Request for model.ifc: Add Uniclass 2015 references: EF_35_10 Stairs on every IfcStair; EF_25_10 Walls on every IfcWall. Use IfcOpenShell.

First a look at what the model holds.

```python
import ifcopenshell

model = ifcopenshell.open("model.ifc")
print(model.schema)
print("classifications:", [c.Name for c in model.by_type("IfcClassification")])
for ifc_class in ("IfcDoor", "IfcRoof", "IfcStair", "IfcWall", "IfcWindow"):
    print(ifc_class, len(model.by_type(ifc_class)))
```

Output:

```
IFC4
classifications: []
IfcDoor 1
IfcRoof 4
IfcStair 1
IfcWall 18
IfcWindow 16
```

```python
import ifcopenshell
import ifcopenshell.api.classification

model = ifcopenshell.open("model.ifc")

system = ifcopenshell.api.classification.add_classification(model, classification="Uniclass 2015")

codes = {
    "IfcStair": ("EF_35_10", "Stairs"),
    "IfcWall": ("EF_25_10", "Walls"),
}
for ifc_class, (code, name) in codes.items():
    products = model.by_type(ifc_class)
    ifcopenshell.api.classification.add_reference(
        model, products=products, classification=system, identification=code, name=name
    )
    print(code, len(products))

model.write("model-out.ifc")
```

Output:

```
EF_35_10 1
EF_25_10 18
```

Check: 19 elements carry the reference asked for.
